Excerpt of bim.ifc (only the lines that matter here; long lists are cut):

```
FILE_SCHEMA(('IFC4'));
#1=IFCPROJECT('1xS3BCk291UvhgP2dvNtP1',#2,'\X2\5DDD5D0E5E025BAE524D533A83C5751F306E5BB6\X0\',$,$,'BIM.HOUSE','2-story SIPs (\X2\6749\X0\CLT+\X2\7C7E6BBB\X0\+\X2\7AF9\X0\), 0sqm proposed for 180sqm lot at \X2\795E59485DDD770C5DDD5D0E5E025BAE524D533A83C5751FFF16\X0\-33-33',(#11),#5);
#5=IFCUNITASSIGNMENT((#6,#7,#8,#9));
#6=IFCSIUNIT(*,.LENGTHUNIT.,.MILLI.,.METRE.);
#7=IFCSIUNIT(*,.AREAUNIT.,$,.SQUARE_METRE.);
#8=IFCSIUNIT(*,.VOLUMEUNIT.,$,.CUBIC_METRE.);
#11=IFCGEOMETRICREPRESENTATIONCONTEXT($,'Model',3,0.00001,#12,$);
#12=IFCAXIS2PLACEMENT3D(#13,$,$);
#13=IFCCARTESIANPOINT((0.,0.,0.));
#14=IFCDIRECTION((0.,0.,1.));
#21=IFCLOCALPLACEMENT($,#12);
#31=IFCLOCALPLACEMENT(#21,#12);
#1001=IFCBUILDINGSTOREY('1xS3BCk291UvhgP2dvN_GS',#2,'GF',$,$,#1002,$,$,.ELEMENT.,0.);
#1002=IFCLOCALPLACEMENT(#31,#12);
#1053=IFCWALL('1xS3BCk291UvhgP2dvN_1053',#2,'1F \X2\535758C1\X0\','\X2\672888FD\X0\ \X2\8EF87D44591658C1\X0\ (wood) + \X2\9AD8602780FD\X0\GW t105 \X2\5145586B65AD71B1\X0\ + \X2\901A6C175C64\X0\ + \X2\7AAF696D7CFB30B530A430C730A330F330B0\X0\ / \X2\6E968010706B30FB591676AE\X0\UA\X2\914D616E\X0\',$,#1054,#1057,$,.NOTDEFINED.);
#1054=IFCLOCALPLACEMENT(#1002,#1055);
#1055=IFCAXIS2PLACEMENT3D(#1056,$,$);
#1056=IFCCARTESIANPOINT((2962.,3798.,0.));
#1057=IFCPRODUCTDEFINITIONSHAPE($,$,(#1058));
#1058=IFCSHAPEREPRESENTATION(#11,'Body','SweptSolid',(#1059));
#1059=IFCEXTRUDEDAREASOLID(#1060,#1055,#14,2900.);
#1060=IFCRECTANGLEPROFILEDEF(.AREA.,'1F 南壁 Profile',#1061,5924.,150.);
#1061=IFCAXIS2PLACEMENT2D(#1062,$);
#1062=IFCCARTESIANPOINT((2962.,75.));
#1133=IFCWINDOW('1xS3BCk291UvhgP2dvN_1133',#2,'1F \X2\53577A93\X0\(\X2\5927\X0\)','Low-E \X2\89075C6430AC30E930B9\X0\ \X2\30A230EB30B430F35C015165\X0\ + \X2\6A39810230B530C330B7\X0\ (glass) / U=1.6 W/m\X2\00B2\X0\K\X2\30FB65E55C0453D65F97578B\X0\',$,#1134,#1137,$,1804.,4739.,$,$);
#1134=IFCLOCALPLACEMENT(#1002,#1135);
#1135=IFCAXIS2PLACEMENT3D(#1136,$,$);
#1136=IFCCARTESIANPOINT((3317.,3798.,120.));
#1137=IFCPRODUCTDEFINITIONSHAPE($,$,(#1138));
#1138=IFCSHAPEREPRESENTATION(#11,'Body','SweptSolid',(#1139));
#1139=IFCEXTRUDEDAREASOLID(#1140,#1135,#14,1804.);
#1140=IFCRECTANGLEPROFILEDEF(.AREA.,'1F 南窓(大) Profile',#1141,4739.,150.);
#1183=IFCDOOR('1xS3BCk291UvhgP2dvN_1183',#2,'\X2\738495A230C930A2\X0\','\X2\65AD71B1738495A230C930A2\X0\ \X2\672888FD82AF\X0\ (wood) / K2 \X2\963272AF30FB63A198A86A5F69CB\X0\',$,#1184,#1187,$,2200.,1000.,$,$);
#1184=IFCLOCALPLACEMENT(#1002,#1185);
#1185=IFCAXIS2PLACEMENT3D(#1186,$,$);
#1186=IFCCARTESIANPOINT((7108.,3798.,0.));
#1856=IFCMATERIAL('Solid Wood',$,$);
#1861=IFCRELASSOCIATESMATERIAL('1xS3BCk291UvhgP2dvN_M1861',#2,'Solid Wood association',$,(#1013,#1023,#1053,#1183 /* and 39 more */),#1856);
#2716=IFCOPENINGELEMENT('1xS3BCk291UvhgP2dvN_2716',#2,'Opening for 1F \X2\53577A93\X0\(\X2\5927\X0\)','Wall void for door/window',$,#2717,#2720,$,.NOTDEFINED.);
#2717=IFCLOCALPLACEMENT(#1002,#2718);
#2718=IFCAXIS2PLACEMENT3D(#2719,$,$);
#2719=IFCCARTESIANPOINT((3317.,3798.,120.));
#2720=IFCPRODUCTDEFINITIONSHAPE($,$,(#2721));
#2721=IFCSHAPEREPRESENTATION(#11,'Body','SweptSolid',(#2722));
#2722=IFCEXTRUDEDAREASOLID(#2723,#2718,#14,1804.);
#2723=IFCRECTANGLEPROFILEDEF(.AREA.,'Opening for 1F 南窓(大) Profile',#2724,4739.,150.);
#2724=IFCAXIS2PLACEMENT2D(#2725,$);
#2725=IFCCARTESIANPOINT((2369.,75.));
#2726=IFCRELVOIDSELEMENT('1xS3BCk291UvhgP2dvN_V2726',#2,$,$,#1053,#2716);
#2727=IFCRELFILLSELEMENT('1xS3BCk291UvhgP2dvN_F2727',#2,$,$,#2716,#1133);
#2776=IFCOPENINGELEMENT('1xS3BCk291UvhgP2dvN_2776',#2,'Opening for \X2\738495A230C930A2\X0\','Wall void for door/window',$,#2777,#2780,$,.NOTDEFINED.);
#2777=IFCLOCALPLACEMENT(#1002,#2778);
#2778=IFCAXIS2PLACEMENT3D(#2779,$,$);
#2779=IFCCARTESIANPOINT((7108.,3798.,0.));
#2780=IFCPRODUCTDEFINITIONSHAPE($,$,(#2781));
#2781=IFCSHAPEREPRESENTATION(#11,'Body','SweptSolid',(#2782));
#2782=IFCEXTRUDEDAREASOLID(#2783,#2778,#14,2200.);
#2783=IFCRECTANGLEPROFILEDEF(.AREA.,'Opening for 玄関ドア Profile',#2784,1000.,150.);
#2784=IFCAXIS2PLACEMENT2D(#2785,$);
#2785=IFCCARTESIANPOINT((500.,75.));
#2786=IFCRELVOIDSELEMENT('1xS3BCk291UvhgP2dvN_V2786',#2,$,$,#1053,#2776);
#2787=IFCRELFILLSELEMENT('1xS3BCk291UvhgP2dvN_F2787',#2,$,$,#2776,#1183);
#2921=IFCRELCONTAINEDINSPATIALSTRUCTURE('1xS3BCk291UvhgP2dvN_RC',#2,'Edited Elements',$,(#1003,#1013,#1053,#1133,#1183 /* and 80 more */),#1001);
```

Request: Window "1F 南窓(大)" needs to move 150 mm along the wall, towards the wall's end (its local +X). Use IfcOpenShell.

```python
import ifcopenshell
import ifcopenshell.api.geometry
import ifcopenshell.util.placement

model = ifcopenshell.open("bim.ifc")

window = model.by_guid("1xS3BCk291UvhgP2dvN_1133")
opening = window.FillsVoids[0].RelatingOpeningElement
wall = opening.VoidsElements[0].RelatingBuildingElement

wall_matrix = ifcopenshell.util.placement.get_local_placement(wall.ObjectPlacement)
shift = wall_matrix[:3, 0] * 150.0
before = ifcopenshell.util.placement.get_local_placement(window.ObjectPlacement)[:3, 3].copy()

# The window is not placed relative to its opening, so move both.
for product in (opening, window):
    matrix = ifcopenshell.util.placement.get_local_placement(product.ObjectPlacement)
    matrix[:3, 3] += shift
    ifcopenshell.api.geometry.edit_object_placement(model, product=product, matrix=matrix, is_si=False)

after = ifcopenshell.util.placement.get_local_placement(window.ObjectPlacement)[:3, 3]
print("window moved by", (after - before).round(3) + 0.0)

model.write("bim-out.ifc")
```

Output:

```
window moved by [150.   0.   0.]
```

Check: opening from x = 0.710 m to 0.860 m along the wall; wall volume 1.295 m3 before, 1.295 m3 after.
